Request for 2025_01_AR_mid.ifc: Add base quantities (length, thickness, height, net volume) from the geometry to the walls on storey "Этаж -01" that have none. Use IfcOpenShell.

First a look at what the model holds.

```python
import ifcopenshell
import ifcopenshell.util.element
import ifcopenshell.util.unit

model = ifcopenshell.open("2025_01_AR_mid.ifc")
print(model.schema)
for unit_type in ("LENGTHUNIT", "AREAUNIT", "VOLUMEUNIT"):
    print(unit_type, ifcopenshell.util.unit.calculate_unit_scale(model, unit_type))
storey = next(s for s in model.by_type("IfcBuildingStorey") if s.Name == "Этаж -01")
walls = [e for e in ifcopenshell.util.element.get_decomposition(storey) if e.is_a("IfcWall")]
for e in sorted(walls, key=lambda e: e.id()):
    print(e.id(), e.is_a(), e.Name, list(ifcopenshell.util.element.get_psets(e, qtos_only=True)), sep=" | ")
```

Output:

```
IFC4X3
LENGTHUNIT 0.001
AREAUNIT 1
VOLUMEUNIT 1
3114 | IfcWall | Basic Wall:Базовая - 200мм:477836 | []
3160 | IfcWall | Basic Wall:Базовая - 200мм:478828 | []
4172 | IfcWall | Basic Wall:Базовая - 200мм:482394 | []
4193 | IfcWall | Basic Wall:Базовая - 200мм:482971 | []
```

```python
import ifcopenshell
import ifcopenshell.api.pset
import ifcopenshell.geom
import ifcopenshell.util.element
import ifcopenshell.util.shape
import ifcopenshell.util.unit

model = ifcopenshell.open("2025_01_AR_mid.ifc")
unit_scale = ifcopenshell.util.unit.calculate_unit_scale(model)
volume_scale = ifcopenshell.util.unit.calculate_unit_scale(model, "VOLUMEUNIT")
settings = ifcopenshell.geom.settings()

storey = next(s for s in model.by_type("IfcBuildingStorey") if s.Name == "Этаж -01")
walls = [e for e in ifcopenshell.util.element.get_decomposition(storey) if e.is_a("IfcWall")]

for e in sorted(walls, key=lambda e: e.id()):
    if ifcopenshell.util.element.get_psets(e, qtos_only=True, should_inherit=False):
        continue
    # Geometry comes back in metres, in the element's own axes.
    shape = ifcopenshell.geom.create_shape(settings, e)
    values = {
        "Length": ifcopenshell.util.shape.get_x(shape.geometry) / unit_scale,
        "Width": ifcopenshell.util.shape.get_y(shape.geometry) / unit_scale,
        "Height": ifcopenshell.util.shape.get_z(shape.geometry) / unit_scale,
        "NetVolume": ifcopenshell.util.shape.get_volume(shape.geometry) / volume_scale,
    }
    qto = ifcopenshell.api.pset.add_qto(model, product=e, name="Qto_WallBaseQuantities")
    ifcopenshell.api.pset.edit_qto(model, qto=qto, properties=values)
    print(e.id(), {k: round(v, 3) for k, v in values.items()})

model.write("2025_01_AR_mid_updated.ifc")
```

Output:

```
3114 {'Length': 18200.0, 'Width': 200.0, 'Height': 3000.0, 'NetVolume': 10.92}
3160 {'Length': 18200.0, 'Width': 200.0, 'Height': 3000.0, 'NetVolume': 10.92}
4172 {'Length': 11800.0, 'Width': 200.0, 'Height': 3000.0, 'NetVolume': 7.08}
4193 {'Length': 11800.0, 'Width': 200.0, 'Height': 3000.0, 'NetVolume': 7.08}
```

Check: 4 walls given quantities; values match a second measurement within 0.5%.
